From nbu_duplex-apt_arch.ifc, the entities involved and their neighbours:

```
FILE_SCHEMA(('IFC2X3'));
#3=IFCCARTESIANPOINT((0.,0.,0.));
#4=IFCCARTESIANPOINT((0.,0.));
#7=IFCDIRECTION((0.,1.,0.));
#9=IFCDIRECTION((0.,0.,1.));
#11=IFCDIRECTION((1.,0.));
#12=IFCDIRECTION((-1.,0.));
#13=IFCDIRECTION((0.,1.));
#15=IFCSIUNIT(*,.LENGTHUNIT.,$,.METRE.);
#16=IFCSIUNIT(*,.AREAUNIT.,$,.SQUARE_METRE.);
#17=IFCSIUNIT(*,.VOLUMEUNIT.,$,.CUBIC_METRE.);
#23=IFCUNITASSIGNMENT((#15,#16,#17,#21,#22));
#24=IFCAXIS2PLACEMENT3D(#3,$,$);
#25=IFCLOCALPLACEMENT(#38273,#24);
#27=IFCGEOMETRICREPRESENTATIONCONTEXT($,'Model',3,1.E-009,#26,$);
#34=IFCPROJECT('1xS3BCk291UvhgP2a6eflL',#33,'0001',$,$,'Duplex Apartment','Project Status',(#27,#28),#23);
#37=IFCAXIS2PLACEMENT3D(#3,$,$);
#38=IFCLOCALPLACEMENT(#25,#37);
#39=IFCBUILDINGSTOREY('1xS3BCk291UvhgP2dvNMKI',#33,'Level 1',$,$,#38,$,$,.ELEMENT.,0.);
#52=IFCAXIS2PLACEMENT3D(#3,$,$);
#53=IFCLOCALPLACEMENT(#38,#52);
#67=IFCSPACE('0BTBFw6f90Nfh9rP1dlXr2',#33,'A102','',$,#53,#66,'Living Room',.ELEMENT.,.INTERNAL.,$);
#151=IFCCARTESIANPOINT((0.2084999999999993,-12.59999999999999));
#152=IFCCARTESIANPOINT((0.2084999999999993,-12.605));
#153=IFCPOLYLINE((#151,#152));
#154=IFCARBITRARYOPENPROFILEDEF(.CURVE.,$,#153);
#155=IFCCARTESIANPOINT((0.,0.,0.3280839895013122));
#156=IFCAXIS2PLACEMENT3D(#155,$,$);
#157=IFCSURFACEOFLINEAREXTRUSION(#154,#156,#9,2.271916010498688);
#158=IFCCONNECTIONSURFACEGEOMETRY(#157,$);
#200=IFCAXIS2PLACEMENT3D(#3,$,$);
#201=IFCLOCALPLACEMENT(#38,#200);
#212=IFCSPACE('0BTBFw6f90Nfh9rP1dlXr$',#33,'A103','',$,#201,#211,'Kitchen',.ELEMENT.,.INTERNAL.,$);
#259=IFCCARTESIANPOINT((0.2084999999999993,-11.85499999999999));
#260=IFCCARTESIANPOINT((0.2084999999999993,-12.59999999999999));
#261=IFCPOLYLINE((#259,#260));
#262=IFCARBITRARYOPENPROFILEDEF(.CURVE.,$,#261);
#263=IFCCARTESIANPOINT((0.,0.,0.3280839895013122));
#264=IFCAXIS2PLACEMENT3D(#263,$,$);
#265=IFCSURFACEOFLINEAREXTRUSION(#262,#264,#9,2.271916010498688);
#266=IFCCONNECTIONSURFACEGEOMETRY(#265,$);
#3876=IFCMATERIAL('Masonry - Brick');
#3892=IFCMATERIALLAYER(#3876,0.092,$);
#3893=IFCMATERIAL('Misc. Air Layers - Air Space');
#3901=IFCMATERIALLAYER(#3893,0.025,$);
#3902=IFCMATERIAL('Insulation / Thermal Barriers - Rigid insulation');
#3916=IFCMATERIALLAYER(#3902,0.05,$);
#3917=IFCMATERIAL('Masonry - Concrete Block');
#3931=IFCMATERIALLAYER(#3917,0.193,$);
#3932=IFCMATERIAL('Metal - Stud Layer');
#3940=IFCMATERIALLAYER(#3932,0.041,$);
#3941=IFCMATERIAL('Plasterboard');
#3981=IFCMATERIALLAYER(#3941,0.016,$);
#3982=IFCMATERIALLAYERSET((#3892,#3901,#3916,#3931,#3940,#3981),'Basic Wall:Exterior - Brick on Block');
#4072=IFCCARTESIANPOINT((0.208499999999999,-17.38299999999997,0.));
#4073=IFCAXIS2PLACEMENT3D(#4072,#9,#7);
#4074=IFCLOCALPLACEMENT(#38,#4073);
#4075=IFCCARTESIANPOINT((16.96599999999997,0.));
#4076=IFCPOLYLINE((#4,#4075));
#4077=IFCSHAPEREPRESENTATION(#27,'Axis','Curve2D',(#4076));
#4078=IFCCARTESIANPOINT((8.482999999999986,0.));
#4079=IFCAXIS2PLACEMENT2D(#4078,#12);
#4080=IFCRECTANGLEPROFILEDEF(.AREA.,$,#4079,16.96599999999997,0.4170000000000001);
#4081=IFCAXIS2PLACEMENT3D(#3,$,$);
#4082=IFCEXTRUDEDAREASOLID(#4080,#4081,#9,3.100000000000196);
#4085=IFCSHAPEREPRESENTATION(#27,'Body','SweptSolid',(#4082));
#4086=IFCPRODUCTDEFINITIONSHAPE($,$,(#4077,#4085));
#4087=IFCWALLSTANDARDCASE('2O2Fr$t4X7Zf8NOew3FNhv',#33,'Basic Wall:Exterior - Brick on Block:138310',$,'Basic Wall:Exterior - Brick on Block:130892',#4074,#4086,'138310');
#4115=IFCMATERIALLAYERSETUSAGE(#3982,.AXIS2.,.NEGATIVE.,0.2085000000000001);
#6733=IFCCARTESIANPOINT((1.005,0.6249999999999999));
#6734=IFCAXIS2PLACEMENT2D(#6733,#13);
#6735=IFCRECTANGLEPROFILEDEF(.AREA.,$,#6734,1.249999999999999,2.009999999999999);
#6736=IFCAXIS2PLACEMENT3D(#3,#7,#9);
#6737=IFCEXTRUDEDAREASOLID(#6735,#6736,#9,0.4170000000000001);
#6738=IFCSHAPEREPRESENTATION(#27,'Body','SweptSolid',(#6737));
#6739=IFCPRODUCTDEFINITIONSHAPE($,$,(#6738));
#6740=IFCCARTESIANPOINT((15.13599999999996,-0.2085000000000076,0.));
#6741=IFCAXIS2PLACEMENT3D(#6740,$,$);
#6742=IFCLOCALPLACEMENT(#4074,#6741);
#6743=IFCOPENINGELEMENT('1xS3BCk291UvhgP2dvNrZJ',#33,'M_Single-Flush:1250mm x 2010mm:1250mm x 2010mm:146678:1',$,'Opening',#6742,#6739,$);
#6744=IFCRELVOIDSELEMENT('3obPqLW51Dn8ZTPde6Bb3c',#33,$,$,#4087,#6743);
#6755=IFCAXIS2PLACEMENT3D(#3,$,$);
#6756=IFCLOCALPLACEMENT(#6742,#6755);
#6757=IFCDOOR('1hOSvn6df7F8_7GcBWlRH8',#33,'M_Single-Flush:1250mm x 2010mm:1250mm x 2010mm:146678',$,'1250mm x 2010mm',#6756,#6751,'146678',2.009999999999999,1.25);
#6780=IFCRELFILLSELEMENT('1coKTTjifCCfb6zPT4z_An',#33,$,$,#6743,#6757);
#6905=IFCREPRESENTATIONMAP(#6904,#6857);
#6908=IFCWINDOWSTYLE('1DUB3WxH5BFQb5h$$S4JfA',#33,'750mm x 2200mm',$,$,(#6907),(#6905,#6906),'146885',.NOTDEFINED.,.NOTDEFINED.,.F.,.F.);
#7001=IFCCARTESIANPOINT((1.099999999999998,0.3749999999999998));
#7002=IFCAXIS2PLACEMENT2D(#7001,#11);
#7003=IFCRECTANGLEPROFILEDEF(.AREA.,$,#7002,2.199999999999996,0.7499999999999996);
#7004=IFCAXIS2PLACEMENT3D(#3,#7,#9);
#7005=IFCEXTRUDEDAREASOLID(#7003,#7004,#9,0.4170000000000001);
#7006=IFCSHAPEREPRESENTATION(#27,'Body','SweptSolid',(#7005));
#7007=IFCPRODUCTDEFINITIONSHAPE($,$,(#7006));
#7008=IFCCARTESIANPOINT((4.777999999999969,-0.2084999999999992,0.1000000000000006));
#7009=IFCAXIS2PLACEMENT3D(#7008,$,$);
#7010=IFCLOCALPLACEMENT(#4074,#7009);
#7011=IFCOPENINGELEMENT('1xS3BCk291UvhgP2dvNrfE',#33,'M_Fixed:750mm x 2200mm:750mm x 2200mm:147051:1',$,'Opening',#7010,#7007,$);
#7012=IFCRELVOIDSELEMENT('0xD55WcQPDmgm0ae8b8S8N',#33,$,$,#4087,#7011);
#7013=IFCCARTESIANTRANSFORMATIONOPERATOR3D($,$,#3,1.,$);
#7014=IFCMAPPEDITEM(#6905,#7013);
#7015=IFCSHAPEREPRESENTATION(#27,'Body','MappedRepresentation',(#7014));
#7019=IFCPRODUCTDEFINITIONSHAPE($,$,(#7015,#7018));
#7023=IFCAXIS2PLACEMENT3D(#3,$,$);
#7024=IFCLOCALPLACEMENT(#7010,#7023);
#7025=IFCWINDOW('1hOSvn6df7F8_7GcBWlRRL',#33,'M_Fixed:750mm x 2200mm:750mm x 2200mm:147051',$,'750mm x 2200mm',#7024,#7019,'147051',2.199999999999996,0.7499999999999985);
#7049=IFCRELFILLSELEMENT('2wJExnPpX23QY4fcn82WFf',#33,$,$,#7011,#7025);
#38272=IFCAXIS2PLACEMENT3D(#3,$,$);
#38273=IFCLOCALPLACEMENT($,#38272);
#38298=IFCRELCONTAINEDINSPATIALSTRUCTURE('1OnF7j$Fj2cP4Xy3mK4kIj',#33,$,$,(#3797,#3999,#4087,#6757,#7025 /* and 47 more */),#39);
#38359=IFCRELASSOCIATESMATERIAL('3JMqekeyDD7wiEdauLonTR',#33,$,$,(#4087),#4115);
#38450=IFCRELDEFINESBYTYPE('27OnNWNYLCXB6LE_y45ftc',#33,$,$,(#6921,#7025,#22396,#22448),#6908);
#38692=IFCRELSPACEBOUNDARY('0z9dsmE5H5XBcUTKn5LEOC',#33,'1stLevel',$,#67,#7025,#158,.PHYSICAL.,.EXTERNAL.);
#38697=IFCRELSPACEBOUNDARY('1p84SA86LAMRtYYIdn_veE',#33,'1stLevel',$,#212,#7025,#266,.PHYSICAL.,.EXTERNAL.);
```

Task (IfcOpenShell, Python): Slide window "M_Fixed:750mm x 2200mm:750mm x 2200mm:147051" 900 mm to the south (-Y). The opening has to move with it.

```python
import numpy as np
import ifcopenshell
import ifcopenshell.api.geometry
import ifcopenshell.util.placement

model = ifcopenshell.open("nbu_duplex-apt_arch.ifc")

window = model.by_guid("1hOSvn6df7F8_7GcBWlRRL")
opening = window.FillsVoids[0].RelatingOpeningElement
wall = opening.VoidsElements[0].RelatingBuildingElement

wall_matrix = ifcopenshell.util.placement.get_local_placement(wall.ObjectPlacement)
shift = wall_matrix[:3, 0] * -0.9
before = ifcopenshell.util.placement.get_local_placement(window.ObjectPlacement)[:3, 3].copy()

# The window is placed relative to its opening, so it follows when the opening moves.
matrix = ifcopenshell.util.placement.get_local_placement(opening.ObjectPlacement)
matrix[:3, 3] += shift
ifcopenshell.api.geometry.edit_object_placement(
    model, product=opening, matrix=matrix, is_si=False, should_transform_children=True
)

# Space boundary surfaces are stored in each space's coordinates; move them too.
for rel in window.ProvidesBoundaries:
    if not rel.ConnectionGeometry:
        continue
    surface = rel.ConnectionGeometry.SurfaceOnRelatingElement
    space_matrix = ifcopenshell.util.placement.get_local_placement(rel.RelatingSpace.ObjectPlacement)
    point = np.array(surface.Position.Location.Coordinates) + space_matrix[:3, :3].T @ shift
    surface.Position = model.createIfcAxis2Placement3D(
        model.createIfcCartesianPoint(point.tolist()), surface.Position.Axis, surface.Position.RefDirection
    )

after = ifcopenshell.util.placement.get_local_placement(window.ObjectPlacement)[:3, 3]
print("window moved by", (after - before).round(3) + 0.0)

model.write("nbu_duplex-apt_arch_edited.ifc")
```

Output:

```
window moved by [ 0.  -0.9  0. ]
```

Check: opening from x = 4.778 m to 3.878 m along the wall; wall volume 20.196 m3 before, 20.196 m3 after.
